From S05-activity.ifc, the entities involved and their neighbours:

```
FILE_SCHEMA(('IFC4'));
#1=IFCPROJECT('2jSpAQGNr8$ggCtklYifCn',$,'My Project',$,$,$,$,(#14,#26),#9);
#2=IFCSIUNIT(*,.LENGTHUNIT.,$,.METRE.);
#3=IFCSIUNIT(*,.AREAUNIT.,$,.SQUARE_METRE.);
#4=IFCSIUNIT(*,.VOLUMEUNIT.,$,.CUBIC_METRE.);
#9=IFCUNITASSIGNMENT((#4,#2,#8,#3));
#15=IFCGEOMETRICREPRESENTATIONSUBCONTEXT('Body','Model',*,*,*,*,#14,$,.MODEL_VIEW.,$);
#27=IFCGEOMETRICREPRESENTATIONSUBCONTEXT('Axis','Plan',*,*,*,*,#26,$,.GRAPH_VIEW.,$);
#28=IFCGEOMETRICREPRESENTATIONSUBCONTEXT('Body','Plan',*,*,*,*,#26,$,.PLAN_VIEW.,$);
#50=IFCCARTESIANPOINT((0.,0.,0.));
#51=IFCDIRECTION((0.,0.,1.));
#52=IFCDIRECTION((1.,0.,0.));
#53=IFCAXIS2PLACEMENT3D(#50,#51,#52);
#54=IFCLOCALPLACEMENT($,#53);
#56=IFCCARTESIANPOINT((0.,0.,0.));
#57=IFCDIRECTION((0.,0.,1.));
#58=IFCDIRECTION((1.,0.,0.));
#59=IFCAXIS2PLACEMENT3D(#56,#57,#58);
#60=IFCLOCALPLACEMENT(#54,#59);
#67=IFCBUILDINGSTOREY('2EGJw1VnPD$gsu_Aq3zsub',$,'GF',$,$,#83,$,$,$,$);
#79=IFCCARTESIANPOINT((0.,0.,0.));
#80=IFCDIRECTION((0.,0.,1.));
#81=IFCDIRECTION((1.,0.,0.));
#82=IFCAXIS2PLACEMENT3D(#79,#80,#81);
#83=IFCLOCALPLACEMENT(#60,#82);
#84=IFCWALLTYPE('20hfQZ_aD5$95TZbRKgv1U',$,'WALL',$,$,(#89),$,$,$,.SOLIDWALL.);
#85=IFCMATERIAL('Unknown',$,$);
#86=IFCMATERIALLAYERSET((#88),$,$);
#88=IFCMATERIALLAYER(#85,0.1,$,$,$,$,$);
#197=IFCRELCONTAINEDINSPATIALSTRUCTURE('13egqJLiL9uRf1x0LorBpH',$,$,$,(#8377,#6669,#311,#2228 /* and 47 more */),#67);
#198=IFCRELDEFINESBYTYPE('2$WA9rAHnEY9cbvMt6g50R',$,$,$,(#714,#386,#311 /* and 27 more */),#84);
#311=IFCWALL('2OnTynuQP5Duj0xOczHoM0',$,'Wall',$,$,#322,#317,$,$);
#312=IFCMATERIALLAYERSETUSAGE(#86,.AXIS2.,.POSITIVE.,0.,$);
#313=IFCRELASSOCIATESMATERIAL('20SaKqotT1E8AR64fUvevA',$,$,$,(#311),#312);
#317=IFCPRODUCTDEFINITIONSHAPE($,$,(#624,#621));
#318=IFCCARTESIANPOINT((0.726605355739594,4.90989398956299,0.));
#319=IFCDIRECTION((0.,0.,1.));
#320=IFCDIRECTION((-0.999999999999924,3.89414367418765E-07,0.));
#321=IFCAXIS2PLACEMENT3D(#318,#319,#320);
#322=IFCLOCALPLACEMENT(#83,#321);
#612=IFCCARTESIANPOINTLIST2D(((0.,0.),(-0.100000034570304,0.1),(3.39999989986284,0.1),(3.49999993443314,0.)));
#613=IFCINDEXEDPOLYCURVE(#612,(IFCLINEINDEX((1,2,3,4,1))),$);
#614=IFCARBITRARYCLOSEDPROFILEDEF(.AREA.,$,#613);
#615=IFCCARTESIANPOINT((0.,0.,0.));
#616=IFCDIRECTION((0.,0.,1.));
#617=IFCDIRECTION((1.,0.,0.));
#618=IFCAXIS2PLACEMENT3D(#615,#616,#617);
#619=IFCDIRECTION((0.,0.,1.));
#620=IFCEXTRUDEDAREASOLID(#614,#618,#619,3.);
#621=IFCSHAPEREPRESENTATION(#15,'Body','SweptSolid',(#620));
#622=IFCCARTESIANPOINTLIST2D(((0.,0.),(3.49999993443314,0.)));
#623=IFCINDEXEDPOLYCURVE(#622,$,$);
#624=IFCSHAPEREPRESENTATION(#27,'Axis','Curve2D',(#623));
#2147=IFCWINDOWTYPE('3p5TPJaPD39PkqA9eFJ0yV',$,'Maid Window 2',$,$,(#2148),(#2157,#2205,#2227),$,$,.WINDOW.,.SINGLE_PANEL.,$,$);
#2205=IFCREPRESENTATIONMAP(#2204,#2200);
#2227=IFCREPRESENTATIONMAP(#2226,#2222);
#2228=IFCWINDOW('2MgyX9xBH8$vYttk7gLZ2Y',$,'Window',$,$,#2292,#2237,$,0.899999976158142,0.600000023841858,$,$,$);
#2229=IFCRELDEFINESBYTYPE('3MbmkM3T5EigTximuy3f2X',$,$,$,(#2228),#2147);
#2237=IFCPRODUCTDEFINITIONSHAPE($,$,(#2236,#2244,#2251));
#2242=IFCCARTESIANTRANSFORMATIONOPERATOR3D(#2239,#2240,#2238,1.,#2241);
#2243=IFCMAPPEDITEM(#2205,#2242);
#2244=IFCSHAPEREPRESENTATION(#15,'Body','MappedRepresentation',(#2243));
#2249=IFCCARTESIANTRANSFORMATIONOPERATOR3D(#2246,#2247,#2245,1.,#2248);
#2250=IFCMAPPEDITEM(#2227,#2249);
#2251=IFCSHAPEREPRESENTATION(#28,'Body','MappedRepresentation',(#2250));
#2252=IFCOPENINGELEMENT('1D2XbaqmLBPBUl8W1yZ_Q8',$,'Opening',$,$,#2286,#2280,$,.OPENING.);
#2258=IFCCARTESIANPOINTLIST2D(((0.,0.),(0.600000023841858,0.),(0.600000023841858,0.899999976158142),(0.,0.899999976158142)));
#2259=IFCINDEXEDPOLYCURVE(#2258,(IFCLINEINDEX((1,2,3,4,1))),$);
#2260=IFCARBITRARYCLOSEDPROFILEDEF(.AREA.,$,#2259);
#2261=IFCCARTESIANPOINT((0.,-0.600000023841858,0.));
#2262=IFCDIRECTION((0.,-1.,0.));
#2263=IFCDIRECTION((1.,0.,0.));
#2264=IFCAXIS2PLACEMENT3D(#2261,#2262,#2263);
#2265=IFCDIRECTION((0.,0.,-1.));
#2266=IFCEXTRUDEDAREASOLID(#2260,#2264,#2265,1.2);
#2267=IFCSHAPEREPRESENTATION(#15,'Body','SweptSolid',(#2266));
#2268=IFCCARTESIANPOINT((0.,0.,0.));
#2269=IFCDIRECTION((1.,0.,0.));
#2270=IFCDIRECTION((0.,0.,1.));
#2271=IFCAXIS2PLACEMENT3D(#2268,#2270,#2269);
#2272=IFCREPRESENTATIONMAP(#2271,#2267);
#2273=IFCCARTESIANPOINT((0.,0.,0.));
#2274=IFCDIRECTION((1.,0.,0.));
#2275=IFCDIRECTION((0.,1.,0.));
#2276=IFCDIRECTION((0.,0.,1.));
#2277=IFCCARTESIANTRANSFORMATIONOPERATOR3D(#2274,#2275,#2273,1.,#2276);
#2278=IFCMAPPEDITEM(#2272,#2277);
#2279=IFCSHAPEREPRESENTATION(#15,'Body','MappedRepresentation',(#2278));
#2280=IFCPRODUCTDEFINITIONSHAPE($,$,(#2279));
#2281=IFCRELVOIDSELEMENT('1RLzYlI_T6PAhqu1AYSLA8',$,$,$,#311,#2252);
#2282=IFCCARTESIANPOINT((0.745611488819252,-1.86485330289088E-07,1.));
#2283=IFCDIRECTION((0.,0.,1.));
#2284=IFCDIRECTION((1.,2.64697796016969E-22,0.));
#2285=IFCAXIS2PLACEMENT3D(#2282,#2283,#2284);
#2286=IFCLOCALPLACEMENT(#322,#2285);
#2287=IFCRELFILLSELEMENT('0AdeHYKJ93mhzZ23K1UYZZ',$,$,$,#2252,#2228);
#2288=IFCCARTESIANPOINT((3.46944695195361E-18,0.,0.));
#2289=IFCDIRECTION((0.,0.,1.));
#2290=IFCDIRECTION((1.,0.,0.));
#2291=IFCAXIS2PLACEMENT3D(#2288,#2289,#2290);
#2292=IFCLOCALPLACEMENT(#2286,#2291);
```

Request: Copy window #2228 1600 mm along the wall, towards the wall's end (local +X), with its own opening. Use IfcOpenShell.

```python
import ifcopenshell
import ifcopenshell.api.feature
import ifcopenshell.api.geometry
import ifcopenshell.api.root
import ifcopenshell.geom
import ifcopenshell.util.element
import ifcopenshell.util.placement
import ifcopenshell.util.shape

model = ifcopenshell.open("S05-activity.ifc")
settings = ifcopenshell.geom.settings()


def volume(element):
    """Net volume in cubic metres, openings subtracted."""
    shape = ifcopenshell.geom.create_shape(settings, element)
    return ifcopenshell.util.shape.get_volume(shape.geometry)


window = model.by_guid("2MgyX9xBH8$vYttk7gLZ2Y")
opening = window.FillsVoids[0].RelatingOpeningElement
wall = opening.VoidsElements[0].RelatingBuildingElement
before = volume(wall)
shift = ifcopenshell.util.placement.get_local_placement(wall.ObjectPlacement)[:3, 0] * 1.6

# copy_class copies the void relationship, type, container and properties, but no geometry.
new_opening = ifcopenshell.api.root.copy_class(model, product=opening)
new_opening.Representation = ifcopenshell.util.element.copy_deep(
    model, opening.Representation, exclude=["IfcGeometricRepresentationContext", "IfcRepresentationMap"]
)
new_window = ifcopenshell.api.root.copy_class(model, product=window)
new_window.Representation = ifcopenshell.util.element.copy_deep(
    model, window.Representation, exclude=["IfcGeometricRepresentationContext", "IfcRepresentationMap"]
)
ifcopenshell.api.feature.add_filling(model, opening=new_opening, element=new_window)

for old, new in ((opening, new_opening), (window, new_window)):
    matrix = ifcopenshell.util.placement.get_local_placement(old.ObjectPlacement)
    matrix[:3, 3] += shift
    ifcopenshell.api.geometry.edit_object_placement(model, product=new, matrix=matrix, is_si=False)

after = volume(wall)

print(f"wall volume {before:.3f} -> {after:.3f} m3")

model.write("S05-activity_v2.ifc")
```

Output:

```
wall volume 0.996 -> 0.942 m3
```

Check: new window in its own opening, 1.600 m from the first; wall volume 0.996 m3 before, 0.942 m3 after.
